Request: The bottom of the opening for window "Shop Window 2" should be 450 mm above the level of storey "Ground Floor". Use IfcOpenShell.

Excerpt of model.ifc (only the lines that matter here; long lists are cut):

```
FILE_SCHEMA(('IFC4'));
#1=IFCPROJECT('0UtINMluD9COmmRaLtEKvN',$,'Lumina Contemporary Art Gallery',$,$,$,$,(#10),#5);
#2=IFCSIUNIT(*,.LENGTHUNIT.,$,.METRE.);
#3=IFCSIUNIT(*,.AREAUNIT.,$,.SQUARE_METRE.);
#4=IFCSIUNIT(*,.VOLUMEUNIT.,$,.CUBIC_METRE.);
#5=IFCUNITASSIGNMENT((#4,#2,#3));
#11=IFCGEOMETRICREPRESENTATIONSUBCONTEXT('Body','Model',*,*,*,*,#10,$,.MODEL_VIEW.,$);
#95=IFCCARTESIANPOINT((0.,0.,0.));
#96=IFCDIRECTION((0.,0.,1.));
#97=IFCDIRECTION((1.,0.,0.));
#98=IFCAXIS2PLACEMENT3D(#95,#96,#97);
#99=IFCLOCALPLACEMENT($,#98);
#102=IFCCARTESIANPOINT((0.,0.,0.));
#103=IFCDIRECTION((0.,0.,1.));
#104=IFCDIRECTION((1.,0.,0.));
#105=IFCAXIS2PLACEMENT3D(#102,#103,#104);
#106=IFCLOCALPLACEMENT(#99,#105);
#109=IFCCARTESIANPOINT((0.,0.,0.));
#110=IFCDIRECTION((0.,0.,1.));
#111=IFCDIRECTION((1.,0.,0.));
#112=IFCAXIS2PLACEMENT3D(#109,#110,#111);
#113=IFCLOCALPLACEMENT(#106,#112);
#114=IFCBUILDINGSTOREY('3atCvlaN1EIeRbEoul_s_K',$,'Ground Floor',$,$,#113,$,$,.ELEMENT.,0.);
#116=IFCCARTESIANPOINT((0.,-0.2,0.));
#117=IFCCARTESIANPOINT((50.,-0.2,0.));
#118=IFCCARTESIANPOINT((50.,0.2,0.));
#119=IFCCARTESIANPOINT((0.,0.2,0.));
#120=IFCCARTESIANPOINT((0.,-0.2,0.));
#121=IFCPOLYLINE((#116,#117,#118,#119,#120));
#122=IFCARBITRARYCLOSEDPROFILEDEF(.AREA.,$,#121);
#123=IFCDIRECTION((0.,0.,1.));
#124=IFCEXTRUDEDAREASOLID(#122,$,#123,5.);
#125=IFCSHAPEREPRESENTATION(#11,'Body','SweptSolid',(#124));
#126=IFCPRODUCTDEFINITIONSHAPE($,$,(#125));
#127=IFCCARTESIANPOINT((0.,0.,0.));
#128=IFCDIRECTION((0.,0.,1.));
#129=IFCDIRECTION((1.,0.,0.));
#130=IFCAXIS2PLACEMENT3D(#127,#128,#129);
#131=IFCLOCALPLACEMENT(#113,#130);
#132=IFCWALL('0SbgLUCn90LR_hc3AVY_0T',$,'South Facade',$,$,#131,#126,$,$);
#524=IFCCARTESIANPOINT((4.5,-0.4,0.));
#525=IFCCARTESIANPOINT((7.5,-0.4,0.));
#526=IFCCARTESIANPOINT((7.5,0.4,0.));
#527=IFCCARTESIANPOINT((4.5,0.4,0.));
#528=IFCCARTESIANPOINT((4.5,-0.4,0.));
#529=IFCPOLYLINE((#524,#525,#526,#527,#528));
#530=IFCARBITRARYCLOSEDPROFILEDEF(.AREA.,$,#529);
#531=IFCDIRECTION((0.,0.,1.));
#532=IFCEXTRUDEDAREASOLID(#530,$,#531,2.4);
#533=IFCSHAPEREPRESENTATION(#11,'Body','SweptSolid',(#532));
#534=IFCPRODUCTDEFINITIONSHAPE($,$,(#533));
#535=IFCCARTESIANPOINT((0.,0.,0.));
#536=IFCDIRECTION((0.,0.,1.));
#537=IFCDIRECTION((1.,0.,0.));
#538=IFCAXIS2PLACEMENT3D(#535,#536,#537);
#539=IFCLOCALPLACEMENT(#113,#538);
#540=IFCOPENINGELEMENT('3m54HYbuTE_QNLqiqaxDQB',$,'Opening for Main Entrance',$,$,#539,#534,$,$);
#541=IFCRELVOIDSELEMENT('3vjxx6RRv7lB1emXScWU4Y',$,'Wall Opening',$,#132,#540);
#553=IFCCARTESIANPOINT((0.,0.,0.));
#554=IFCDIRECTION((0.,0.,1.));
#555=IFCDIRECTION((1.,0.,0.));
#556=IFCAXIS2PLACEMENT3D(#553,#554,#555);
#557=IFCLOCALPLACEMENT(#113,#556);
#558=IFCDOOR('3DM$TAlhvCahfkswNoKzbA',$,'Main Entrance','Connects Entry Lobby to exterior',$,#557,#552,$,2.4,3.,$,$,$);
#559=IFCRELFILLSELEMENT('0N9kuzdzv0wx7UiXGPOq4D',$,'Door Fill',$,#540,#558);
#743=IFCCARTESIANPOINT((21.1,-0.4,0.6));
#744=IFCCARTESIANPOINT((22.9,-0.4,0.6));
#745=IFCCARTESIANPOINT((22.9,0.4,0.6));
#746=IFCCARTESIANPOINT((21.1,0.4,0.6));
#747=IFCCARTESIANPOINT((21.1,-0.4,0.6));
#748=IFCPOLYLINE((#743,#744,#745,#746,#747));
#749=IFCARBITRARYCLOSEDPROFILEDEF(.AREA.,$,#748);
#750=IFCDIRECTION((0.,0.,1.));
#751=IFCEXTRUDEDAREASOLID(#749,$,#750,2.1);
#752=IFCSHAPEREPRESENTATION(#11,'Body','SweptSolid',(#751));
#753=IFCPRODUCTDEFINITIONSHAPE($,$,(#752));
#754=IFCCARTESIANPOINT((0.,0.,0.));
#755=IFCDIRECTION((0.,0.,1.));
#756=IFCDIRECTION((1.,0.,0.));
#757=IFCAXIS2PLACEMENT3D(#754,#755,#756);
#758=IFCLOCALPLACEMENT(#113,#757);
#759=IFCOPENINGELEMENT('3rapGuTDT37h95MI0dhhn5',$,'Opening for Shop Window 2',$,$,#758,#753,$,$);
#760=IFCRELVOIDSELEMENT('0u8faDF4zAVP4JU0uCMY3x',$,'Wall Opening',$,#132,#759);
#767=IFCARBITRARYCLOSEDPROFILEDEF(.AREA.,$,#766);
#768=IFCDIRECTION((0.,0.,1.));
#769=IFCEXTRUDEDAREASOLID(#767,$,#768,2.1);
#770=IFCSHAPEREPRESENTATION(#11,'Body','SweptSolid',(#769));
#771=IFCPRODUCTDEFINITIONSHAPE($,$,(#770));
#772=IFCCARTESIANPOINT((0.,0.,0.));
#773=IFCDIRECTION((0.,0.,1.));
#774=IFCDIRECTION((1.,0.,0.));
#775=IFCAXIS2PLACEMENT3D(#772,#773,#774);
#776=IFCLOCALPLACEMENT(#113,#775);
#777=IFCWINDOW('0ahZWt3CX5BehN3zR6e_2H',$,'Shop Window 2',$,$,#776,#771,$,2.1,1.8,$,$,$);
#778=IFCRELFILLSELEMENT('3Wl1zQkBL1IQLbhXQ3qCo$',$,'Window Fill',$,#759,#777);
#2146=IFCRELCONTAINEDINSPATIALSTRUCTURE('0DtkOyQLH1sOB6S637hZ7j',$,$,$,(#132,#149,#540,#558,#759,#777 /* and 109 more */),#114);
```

```python
import numpy as np
import ifcopenshell
import ifcopenshell.api.geometry
import ifcopenshell.geom
import ifcopenshell.util.element
import ifcopenshell.util.placement
import ifcopenshell.util.shape
import ifcopenshell.util.unit

model = ifcopenshell.open("model.ifc")
unit_scale = ifcopenshell.util.unit.calculate_unit_scale(model)

window = model.by_guid("0ahZWt3CX5BehN3zR6e_2H")
opening = window.FillsVoids[0].RelatingOpeningElement
storey = ifcopenshell.util.element.get_container(window, ifc_class="IfcBuildingStorey")
level = ifcopenshell.util.placement.get_local_placement(storey.ObjectPlacement)[2, 3]

# The opening's origin need not be at the sill, so measure its lowest point.
shape = ifcopenshell.geom.create_shape(ifcopenshell.geom.settings(), opening)
bottom = ifcopenshell.util.shape.get_shape_bottom_elevation(shape, shape.geometry) / unit_scale
dz = level + 0.45 - bottom

shift = np.array([0.0, 0.0, dz])
# The window is not placed relative to its opening, so move both.
for product in (opening, window):
    matrix = ifcopenshell.util.placement.get_local_placement(product.ObjectPlacement)
    matrix[:3, 3] += shift
    ifcopenshell.api.geometry.edit_object_placement(model, product=product, matrix=matrix, is_si=False)

print(f"moved by {dz * unit_scale:+.3f} m")

model.write("model_edited.ifc")
```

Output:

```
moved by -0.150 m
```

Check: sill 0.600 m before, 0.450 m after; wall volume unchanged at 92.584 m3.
